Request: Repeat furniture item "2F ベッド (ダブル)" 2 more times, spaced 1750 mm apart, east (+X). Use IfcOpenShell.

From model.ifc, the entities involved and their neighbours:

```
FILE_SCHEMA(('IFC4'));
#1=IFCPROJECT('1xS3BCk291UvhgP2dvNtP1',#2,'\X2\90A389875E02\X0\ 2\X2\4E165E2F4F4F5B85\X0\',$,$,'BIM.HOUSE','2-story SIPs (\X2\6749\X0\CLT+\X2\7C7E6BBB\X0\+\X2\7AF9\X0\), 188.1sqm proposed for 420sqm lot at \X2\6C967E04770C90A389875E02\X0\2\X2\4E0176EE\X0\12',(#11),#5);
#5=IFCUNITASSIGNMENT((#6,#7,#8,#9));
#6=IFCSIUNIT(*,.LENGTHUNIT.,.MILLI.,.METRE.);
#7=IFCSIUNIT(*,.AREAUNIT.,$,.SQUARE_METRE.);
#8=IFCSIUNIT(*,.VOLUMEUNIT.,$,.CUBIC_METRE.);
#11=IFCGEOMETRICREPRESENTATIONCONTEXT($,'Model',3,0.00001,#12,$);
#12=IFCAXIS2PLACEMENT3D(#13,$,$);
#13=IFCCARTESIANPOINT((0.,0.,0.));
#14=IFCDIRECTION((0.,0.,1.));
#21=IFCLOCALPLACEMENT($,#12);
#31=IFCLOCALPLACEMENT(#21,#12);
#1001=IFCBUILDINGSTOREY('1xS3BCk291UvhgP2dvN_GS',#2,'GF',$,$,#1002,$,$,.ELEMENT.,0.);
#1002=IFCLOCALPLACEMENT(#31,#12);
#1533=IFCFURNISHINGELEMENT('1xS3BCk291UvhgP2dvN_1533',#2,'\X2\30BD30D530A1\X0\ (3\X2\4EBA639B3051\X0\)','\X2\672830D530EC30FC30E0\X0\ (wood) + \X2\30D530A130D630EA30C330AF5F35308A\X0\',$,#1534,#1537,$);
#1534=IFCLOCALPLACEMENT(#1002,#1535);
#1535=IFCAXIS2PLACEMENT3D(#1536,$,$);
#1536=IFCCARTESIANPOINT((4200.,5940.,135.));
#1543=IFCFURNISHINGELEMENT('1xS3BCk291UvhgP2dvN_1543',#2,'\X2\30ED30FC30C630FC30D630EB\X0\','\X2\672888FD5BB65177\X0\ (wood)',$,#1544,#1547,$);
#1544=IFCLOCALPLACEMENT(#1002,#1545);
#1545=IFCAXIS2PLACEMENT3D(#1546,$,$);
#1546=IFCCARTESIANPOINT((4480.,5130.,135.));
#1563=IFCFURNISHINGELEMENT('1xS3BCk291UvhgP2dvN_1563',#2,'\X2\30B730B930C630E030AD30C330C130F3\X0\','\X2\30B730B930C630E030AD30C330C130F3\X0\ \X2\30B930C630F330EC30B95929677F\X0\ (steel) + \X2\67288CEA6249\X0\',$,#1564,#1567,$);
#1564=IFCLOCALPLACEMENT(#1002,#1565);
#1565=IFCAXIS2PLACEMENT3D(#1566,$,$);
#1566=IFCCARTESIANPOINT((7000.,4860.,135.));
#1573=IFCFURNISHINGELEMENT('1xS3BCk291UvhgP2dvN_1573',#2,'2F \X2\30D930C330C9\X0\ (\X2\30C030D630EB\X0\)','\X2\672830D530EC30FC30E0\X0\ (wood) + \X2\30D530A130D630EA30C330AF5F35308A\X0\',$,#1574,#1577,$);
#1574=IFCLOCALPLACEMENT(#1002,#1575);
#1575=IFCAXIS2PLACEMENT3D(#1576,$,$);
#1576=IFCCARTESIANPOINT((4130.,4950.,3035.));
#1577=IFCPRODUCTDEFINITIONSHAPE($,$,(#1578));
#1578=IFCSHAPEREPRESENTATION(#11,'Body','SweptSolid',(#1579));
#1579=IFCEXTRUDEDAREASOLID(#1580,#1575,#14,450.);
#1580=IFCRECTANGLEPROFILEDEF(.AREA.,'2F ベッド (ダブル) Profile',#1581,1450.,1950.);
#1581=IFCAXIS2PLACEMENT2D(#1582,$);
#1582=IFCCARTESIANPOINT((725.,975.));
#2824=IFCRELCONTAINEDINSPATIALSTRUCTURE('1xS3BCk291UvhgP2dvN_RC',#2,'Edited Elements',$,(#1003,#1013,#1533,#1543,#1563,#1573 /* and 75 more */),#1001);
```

```python
import numpy as np
import ifcopenshell
import ifcopenshell.api.geometry
import ifcopenshell.api.root
import ifcopenshell.util.element
import ifcopenshell.util.placement
import ifcopenshell.util.unit

model = ifcopenshell.open("model.ifc")
unit_scale = ifcopenshell.util.unit.calculate_unit_scale(model)


def reuse_history(source, copy):
    """copy_class also copies each property set's owner history, people and application; keep the originals."""
    for rel in copy.IsDefinedBy:
        if rel.is_a("IfcRelDefinesByProperties") and (history := rel.RelatingPropertyDefinition.OwnerHistory):
            rel.RelatingPropertyDefinition.OwnerHistory = source.OwnerHistory
            ifcopenshell.util.element.remove_deep2(model, history)


source = model.by_guid("1xS3BCk291UvhgP2dvN_1573")
base = ifcopenshell.util.placement.get_local_placement(source.ObjectPlacement)
step = np.array([1.0, 0.0, 0.0]) * 1.75 / unit_scale

for i in range(1, 3):
    copy = ifcopenshell.api.root.copy_class(model, product=source)
    copy.Representation = ifcopenshell.util.element.copy_deep(
        model, source.Representation, exclude=["IfcGeometricRepresentationContext", "IfcRepresentationMap"]
    )
    reuse_history(source, copy)
    matrix = base.copy()
    matrix[:3, 3] += i * step
    print("added at", matrix[:3, 3].round(3) + 0.0)
    ifcopenshell.api.geometry.edit_object_placement(model, product=copy, matrix=matrix, is_si=False)

model.write("model_v2.ifc")
```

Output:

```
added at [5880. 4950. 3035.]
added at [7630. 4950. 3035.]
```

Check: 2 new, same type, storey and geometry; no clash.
